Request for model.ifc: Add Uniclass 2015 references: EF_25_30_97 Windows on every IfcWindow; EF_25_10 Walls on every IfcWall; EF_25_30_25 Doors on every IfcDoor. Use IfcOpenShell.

First a look at what the model holds.

```python
import ifcopenshell

model = ifcopenshell.open("model.ifc")
print(model.schema)
print("classifications:", [c.Name for c in model.by_type("IfcClassification")])
for ifc_class in ("IfcDoor", "IfcRoof", "IfcStair", "IfcWall", "IfcWindow"):
    print(ifc_class, len(model.by_type(ifc_class)))
```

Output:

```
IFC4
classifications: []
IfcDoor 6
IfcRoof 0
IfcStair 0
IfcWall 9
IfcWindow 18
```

```python
import ifcopenshell
import ifcopenshell.api.classification

model = ifcopenshell.open("model.ifc")

system = ifcopenshell.api.classification.add_classification(model, classification="Uniclass 2015")

codes = {
    "IfcWindow": ("EF_25_30_97", "Windows"),
    "IfcWall": ("EF_25_10", "Walls"),
    "IfcDoor": ("EF_25_30_25", "Doors"),
}
for ifc_class, (code, name) in codes.items():
    products = model.by_type(ifc_class)
    ifcopenshell.api.classification.add_reference(
        model, products=products, classification=system, identification=code, name=name
    )
    print(code, len(products))

model.write("model_v2.ifc")
```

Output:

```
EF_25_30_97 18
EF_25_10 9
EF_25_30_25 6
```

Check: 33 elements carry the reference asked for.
